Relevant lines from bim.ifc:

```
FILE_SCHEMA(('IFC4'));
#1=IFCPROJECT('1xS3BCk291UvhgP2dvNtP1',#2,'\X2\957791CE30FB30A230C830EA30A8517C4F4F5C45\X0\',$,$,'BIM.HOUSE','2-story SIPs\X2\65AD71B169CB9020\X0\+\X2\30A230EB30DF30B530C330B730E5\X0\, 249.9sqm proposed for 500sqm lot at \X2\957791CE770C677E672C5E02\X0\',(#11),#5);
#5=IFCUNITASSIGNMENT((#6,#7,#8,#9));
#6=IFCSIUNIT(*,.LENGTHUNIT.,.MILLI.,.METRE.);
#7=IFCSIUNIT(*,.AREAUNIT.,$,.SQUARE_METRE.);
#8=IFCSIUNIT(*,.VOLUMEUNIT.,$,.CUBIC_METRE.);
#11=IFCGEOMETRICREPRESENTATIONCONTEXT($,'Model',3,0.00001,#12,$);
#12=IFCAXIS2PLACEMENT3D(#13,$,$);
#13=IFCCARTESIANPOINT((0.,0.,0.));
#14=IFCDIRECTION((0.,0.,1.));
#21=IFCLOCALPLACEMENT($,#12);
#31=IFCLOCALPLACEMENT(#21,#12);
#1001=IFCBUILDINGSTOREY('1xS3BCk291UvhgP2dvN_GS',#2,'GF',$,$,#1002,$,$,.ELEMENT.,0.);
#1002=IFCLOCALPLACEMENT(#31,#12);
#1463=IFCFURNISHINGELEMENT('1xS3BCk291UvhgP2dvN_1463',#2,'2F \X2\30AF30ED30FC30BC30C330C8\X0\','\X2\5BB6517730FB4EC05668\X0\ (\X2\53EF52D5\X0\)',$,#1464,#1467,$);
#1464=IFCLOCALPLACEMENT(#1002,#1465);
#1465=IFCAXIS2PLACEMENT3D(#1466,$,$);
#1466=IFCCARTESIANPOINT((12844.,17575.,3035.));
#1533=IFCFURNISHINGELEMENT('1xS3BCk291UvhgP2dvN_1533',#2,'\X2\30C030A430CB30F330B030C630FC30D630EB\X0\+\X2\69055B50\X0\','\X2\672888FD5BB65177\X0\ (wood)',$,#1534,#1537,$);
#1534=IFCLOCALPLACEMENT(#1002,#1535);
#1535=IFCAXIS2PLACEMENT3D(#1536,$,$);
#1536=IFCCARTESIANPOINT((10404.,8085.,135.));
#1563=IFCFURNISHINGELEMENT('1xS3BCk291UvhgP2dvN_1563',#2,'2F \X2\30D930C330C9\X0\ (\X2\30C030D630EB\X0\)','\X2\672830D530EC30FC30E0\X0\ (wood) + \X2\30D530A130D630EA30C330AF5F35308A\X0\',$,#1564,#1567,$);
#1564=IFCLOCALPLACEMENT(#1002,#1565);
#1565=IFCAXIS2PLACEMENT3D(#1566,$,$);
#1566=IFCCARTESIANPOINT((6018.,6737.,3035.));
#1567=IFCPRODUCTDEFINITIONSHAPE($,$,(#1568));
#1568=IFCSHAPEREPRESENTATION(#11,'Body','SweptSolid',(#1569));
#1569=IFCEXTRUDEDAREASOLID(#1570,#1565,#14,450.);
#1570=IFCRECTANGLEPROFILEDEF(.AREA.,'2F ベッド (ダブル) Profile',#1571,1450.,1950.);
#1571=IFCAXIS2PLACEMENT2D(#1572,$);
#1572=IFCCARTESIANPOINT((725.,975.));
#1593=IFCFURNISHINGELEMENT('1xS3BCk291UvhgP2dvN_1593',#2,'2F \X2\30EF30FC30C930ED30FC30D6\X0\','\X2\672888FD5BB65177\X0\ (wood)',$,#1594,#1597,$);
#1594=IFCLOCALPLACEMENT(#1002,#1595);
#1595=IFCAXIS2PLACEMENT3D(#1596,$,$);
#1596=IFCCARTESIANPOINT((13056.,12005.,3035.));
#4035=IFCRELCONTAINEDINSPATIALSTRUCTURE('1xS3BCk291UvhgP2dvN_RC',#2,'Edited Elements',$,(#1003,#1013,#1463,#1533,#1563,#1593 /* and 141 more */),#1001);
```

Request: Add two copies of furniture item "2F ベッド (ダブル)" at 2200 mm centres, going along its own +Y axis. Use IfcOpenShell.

```python
import ifcopenshell
import ifcopenshell.api.geometry
import ifcopenshell.api.root
import ifcopenshell.util.element
import ifcopenshell.util.placement
import ifcopenshell.util.unit

model = ifcopenshell.open("bim.ifc")
unit_scale = ifcopenshell.util.unit.calculate_unit_scale(model)


def reuse_history(source, copy):
    """copy_class also copies each property set's owner history, people and application; keep the originals."""
    for rel in copy.IsDefinedBy:
        if rel.is_a("IfcRelDefinesByProperties") and (history := rel.RelatingPropertyDefinition.OwnerHistory):
            rel.RelatingPropertyDefinition.OwnerHistory = source.OwnerHistory
            ifcopenshell.util.element.remove_deep2(model, history)


source = model.by_guid("1xS3BCk291UvhgP2dvN_1563")
base = ifcopenshell.util.placement.get_local_placement(source.ObjectPlacement)
step = base[:3, 1] * 2.2 / unit_scale

for i in range(1, 3):
    copy = ifcopenshell.api.root.copy_class(model, product=source)
    copy.Representation = ifcopenshell.util.element.copy_deep(
        model, source.Representation, exclude=["IfcGeometricRepresentationContext", "IfcRepresentationMap"]
    )
    reuse_history(source, copy)
    matrix = base.copy()
    matrix[:3, 3] += i * step
    print("added at", matrix[:3, 3].round(3) + 0.0)
    ifcopenshell.api.geometry.edit_object_placement(model, product=copy, matrix=matrix, is_si=False)

model.write("bim_edited.ifc")
```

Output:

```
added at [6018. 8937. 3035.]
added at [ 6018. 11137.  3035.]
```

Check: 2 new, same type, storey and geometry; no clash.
